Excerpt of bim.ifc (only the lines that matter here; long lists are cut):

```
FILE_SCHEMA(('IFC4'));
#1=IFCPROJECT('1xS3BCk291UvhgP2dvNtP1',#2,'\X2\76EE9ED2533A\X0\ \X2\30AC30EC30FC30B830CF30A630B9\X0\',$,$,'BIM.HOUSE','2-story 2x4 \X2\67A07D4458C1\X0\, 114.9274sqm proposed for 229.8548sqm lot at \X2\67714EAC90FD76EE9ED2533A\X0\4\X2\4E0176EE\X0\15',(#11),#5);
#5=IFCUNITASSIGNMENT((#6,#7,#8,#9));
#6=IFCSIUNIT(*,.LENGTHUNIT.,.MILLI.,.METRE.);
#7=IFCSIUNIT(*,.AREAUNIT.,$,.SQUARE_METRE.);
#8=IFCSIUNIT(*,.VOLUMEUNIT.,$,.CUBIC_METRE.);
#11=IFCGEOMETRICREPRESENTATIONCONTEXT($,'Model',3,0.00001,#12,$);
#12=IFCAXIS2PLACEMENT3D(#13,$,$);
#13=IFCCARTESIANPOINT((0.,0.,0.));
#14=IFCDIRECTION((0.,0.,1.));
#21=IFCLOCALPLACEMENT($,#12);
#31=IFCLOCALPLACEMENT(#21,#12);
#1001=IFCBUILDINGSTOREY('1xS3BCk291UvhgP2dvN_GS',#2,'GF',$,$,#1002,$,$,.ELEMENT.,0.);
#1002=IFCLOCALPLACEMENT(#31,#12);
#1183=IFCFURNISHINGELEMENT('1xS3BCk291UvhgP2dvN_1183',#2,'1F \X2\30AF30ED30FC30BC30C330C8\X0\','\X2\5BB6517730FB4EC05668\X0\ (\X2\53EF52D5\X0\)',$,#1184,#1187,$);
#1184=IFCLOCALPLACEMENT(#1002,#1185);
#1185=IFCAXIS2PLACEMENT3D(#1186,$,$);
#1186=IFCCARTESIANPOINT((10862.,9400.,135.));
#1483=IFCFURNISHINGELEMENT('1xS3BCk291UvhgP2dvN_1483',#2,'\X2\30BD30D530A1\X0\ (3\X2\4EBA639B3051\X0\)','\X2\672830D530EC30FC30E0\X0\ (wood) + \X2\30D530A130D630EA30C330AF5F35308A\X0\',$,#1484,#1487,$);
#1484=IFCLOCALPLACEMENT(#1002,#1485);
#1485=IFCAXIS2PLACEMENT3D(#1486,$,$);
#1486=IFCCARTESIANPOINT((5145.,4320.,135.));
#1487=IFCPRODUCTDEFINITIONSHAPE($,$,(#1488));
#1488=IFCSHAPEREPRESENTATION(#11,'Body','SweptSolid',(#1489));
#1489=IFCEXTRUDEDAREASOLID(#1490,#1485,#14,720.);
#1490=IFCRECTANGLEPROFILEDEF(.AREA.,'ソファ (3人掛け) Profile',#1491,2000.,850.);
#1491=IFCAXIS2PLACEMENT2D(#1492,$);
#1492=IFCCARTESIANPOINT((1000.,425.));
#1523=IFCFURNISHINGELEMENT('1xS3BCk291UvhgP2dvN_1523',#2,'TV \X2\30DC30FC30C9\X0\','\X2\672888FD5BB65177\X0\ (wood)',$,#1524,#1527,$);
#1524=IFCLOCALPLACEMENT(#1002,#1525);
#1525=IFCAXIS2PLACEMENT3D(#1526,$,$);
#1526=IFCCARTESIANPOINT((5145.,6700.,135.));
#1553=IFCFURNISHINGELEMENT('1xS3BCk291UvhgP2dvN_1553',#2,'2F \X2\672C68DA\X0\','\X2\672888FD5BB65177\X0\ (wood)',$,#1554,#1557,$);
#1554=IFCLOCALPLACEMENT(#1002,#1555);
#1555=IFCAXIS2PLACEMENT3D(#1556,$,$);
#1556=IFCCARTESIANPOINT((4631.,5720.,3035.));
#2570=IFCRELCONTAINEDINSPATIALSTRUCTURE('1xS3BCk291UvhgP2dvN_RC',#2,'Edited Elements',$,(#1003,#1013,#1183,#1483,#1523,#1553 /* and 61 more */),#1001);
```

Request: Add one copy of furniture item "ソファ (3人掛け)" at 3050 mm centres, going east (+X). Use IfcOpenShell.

```python
import numpy as np
import ifcopenshell
import ifcopenshell.api.geometry
import ifcopenshell.api.root
import ifcopenshell.util.element
import ifcopenshell.util.placement
import ifcopenshell.util.unit

model = ifcopenshell.open("bim.ifc")
unit_scale = ifcopenshell.util.unit.calculate_unit_scale(model)


def reuse_history(source, copy):
    """copy_class also copies each property set's owner history, people and application; keep the originals."""
    for rel in copy.IsDefinedBy:
        if rel.is_a("IfcRelDefinesByProperties") and (history := rel.RelatingPropertyDefinition.OwnerHistory):
            rel.RelatingPropertyDefinition.OwnerHistory = source.OwnerHistory
            ifcopenshell.util.element.remove_deep2(model, history)


source = model.by_id(1483)
base = ifcopenshell.util.placement.get_local_placement(source.ObjectPlacement)
step = np.array([1.0, 0.0, 0.0]) * 3.05 / unit_scale

for i in range(1, 2):
    copy = ifcopenshell.api.root.copy_class(model, product=source)
    copy.Representation = ifcopenshell.util.element.copy_deep(
        model, source.Representation, exclude=["IfcGeometricRepresentationContext", "IfcRepresentationMap"]
    )
    reuse_history(source, copy)
    matrix = base.copy()
    matrix[:3, 3] += i * step
    print("added at", matrix[:3, 3].round(3) + 0.0)
    ifcopenshell.api.geometry.edit_object_placement(model, product=copy, matrix=matrix, is_si=False)

model.write("bim_updated.ifc")
```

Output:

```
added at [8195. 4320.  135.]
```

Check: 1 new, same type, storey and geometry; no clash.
